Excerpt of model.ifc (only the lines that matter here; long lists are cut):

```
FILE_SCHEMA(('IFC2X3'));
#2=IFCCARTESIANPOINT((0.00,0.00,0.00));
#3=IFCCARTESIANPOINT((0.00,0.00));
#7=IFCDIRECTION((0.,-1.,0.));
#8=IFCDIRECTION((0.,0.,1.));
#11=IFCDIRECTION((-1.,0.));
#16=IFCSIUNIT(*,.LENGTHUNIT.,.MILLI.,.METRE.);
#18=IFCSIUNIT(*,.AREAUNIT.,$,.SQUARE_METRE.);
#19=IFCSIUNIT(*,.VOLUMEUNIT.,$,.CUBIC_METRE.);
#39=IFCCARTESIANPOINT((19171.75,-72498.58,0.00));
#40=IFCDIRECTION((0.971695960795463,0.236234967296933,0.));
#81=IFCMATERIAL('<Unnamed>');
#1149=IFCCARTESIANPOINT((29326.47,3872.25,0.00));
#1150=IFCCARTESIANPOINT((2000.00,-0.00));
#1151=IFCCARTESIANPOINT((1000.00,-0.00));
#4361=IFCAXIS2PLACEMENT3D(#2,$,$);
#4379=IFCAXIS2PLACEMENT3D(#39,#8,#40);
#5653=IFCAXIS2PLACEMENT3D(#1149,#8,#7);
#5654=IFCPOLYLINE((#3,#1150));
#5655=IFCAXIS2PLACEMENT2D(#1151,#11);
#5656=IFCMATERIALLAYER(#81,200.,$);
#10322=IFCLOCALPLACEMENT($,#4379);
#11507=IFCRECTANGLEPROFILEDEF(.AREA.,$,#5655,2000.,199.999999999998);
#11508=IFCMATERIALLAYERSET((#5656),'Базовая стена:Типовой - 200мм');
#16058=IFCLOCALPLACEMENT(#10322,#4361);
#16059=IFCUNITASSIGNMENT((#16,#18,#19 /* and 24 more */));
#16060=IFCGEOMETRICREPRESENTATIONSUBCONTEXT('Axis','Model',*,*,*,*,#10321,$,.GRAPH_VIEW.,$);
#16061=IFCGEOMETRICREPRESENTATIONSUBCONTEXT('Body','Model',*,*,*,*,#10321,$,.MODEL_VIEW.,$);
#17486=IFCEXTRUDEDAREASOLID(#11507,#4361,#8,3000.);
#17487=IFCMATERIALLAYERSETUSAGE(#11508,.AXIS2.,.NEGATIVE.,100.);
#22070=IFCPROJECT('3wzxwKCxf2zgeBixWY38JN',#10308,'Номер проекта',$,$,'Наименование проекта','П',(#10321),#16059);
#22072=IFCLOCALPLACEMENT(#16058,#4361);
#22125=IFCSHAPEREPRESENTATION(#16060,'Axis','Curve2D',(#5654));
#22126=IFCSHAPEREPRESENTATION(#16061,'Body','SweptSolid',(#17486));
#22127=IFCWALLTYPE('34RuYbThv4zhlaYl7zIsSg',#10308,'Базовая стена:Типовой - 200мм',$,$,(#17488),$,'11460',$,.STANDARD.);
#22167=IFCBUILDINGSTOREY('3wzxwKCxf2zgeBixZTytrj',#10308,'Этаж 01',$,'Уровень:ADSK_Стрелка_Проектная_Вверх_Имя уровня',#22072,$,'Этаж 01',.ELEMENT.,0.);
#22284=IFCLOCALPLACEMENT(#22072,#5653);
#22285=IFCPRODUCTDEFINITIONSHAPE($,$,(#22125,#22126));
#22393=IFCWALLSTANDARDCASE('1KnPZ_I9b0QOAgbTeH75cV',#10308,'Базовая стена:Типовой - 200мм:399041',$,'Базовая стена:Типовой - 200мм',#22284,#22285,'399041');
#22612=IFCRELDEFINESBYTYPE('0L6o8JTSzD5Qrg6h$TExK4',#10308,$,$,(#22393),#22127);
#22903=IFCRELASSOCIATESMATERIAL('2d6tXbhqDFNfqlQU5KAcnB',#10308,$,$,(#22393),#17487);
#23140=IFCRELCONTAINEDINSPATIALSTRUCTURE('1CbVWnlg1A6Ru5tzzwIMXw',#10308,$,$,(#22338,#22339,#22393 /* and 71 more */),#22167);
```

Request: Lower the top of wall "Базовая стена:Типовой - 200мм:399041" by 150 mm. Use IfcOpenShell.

```python
import ifcopenshell
import ifcopenshell.geom
import ifcopenshell.util.representation
import ifcopenshell.util.shape
import ifcopenshell.util.unit

model = ifcopenshell.open("model.ifc")
unit_scale = ifcopenshell.util.unit.calculate_unit_scale(model)
settings = ifcopenshell.geom.settings()


def volume(element):
    """Net volume in cubic metres, openings subtracted."""
    shape = ifcopenshell.geom.create_shape(settings, element)
    return ifcopenshell.util.shape.get_volume(shape.geometry)


wall = model.by_guid("1KnPZ_I9b0QOAgbTeH75cV")
before = volume(wall)

body = ifcopenshell.util.representation.get_representation(wall, "Model", "Body")
solid = body.Items[0]
old_height = solid.Depth
solid.Depth -= 0.15 / unit_scale
after = volume(wall)

print(f"height {old_height:g} -> {solid.Depth:g}, volume {before:.3f} -> {after:.3f} m3")

model.write("model-out.ifc")
```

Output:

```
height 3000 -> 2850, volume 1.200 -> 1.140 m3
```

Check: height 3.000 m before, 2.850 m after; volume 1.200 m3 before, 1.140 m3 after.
